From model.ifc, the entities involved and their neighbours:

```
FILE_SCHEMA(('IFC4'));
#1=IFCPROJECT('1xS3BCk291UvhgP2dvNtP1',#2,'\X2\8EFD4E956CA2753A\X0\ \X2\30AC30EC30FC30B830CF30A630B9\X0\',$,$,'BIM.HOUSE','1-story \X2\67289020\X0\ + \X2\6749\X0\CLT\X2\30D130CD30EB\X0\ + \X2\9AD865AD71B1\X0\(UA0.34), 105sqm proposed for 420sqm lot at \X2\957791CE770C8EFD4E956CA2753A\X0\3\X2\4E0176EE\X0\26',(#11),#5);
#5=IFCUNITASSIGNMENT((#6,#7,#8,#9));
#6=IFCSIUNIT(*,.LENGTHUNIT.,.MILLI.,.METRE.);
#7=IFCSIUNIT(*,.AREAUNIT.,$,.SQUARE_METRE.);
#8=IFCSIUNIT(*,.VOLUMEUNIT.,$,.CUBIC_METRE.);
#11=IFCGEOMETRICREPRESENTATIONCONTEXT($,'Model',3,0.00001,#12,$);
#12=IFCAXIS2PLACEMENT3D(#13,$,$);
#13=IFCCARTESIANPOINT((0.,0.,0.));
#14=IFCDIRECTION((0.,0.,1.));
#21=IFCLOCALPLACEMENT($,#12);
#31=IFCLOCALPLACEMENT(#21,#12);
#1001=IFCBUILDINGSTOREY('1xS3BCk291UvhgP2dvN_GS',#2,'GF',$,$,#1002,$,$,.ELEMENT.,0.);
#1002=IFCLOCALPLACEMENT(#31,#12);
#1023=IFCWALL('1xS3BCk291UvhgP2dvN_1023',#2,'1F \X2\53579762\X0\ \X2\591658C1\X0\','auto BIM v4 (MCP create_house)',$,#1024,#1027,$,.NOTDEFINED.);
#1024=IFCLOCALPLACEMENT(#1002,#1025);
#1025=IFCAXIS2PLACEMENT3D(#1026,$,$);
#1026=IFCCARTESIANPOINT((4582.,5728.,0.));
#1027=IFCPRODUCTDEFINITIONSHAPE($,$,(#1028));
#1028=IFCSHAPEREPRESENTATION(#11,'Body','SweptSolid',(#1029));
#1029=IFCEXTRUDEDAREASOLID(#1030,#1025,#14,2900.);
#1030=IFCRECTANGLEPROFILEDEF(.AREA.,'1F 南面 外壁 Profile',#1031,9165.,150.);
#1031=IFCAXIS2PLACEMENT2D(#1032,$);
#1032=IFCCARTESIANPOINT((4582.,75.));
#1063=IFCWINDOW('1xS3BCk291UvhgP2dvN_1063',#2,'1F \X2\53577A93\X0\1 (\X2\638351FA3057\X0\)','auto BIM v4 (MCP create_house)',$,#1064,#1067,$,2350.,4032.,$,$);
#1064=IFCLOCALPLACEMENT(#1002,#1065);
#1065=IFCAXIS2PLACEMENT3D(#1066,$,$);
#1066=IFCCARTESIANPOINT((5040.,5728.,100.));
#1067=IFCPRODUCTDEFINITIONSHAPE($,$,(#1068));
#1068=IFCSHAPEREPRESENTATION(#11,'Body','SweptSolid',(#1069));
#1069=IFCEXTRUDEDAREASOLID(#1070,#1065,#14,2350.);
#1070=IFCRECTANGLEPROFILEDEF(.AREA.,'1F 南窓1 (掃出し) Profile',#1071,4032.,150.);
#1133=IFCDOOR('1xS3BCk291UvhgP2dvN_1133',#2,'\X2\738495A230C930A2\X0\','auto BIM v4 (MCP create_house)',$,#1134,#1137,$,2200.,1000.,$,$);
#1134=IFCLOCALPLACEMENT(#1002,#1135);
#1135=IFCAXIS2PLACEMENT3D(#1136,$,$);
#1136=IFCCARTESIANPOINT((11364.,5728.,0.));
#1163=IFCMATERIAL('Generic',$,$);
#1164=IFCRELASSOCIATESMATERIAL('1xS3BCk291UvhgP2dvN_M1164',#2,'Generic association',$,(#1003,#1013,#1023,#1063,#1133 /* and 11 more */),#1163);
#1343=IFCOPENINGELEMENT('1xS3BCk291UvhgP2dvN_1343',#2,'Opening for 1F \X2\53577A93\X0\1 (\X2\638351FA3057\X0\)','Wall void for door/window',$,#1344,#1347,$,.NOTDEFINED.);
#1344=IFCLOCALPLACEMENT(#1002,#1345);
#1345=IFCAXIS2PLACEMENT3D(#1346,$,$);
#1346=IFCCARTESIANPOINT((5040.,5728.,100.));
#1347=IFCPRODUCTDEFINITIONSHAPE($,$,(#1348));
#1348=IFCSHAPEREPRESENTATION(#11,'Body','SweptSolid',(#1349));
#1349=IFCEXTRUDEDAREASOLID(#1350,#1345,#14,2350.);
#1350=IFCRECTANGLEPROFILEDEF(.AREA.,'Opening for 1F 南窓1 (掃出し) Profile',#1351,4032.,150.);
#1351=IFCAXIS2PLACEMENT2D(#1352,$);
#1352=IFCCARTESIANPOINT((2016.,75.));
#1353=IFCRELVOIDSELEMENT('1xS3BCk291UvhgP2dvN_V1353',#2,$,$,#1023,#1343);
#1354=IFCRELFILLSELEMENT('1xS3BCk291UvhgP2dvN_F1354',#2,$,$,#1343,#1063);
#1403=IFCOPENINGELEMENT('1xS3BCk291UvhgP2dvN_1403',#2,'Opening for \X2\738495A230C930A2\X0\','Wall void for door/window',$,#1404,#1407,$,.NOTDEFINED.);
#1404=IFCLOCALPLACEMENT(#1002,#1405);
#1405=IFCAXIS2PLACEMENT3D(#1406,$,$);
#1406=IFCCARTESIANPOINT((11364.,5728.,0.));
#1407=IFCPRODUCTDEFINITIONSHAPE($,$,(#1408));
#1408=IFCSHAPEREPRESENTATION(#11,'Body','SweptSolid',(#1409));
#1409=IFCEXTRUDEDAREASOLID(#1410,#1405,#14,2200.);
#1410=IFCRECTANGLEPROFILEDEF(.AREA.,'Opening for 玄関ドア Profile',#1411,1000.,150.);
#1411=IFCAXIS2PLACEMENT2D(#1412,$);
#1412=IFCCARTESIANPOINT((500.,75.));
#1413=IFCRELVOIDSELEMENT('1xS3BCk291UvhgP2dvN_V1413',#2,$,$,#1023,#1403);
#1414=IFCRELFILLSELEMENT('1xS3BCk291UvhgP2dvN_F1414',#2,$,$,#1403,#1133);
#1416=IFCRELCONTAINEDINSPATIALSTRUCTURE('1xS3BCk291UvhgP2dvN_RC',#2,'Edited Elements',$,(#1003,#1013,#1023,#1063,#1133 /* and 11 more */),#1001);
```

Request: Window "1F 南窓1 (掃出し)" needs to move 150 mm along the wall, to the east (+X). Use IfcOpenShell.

```python
import ifcopenshell
import ifcopenshell.api.geometry
import ifcopenshell.util.placement
import ifcopenshell.util.unit

model = ifcopenshell.open("model.ifc")
unit_scale = ifcopenshell.util.unit.calculate_unit_scale(model)

window = model.by_id(1063)
opening = window.FillsVoids[0].RelatingOpeningElement
wall = opening.VoidsElements[0].RelatingBuildingElement

wall_matrix = ifcopenshell.util.placement.get_local_placement(wall.ObjectPlacement)
shift = wall_matrix[:3, 0] * 0.15 / unit_scale
before = ifcopenshell.util.placement.get_local_placement(window.ObjectPlacement)[:3, 3].copy()

# The window is not placed relative to its opening, so move both.
for product in (opening, window):
    matrix = ifcopenshell.util.placement.get_local_placement(product.ObjectPlacement)
    matrix[:3, 3] += shift
    ifcopenshell.api.geometry.edit_object_placement(model, product=product, matrix=matrix, is_si=False)

after = ifcopenshell.util.placement.get_local_placement(window.ObjectPlacement)[:3, 3]
print("window moved by", (after - before).round(3) + 0.0)

model.write("model_edited.ifc")
```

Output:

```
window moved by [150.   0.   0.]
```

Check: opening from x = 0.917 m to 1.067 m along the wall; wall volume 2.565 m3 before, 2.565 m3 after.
